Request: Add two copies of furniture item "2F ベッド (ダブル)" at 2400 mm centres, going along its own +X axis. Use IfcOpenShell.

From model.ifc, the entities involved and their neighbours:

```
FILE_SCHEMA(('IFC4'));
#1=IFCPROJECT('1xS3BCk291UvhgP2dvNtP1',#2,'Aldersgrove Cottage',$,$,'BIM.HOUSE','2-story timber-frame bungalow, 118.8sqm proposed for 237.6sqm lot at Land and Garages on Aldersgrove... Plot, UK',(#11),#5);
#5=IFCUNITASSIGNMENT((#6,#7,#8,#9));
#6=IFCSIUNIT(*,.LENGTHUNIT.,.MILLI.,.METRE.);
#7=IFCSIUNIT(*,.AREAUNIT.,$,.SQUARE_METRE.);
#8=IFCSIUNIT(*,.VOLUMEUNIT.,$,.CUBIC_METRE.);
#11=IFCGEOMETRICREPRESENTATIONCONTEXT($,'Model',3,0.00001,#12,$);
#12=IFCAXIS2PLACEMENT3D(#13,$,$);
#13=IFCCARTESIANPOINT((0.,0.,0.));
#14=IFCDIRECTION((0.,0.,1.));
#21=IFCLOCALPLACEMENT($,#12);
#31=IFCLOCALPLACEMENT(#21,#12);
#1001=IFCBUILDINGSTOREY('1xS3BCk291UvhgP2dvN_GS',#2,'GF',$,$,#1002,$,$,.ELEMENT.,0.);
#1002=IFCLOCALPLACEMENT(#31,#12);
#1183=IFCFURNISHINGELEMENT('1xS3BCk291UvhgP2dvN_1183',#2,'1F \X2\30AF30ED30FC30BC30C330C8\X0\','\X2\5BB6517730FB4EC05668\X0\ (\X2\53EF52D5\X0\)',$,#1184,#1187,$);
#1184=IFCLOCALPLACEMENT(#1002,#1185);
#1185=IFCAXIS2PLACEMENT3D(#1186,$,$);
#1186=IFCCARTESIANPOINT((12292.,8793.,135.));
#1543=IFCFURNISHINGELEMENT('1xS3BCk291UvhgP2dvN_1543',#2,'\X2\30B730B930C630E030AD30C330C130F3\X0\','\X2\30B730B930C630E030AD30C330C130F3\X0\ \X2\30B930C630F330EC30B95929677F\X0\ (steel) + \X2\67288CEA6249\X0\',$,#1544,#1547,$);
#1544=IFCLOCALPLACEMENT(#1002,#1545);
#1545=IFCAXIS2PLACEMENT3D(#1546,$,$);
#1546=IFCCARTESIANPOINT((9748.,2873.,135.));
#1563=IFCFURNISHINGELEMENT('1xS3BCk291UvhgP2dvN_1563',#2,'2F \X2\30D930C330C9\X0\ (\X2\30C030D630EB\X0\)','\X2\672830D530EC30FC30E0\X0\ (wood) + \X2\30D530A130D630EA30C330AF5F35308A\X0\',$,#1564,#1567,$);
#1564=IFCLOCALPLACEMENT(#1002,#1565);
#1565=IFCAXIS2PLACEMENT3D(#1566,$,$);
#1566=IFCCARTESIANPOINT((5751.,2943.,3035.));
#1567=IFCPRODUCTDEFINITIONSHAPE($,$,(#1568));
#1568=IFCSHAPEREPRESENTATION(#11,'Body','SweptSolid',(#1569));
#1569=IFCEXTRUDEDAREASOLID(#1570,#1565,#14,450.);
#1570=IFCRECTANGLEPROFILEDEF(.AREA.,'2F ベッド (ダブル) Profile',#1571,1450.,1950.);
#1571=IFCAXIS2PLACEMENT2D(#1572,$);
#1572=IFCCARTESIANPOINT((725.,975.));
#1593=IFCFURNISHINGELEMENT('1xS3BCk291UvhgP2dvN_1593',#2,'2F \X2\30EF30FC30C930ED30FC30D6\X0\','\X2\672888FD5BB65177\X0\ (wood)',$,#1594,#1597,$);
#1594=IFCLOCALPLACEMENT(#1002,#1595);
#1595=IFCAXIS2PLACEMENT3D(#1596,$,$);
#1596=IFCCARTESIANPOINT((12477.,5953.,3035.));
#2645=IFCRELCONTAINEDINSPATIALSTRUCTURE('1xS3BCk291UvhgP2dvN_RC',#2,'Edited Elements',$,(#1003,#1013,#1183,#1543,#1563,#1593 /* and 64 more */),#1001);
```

```python
import ifcopenshell
import ifcopenshell.api.geometry
import ifcopenshell.api.root
import ifcopenshell.util.element
import ifcopenshell.util.placement

model = ifcopenshell.open("model.ifc")


def reuse_history(source, copy):
    """copy_class also copies each property set's owner history, people and application; keep the originals."""
    for rel in copy.IsDefinedBy:
        if rel.is_a("IfcRelDefinesByProperties") and (history := rel.RelatingPropertyDefinition.OwnerHistory):
            rel.RelatingPropertyDefinition.OwnerHistory = source.OwnerHistory
            ifcopenshell.util.element.remove_deep2(model, history)


source = model.by_guid("1xS3BCk291UvhgP2dvN_1563")
base = ifcopenshell.util.placement.get_local_placement(source.ObjectPlacement)
step = base[:3, 0] * 2400.0

for i in range(1, 3):
    copy = ifcopenshell.api.root.copy_class(model, product=source)
    copy.Representation = ifcopenshell.util.element.copy_deep(
        model, source.Representation, exclude=["IfcGeometricRepresentationContext", "IfcRepresentationMap"]
    )
    reuse_history(source, copy)
    matrix = base.copy()
    matrix[:3, 3] += i * step
    print("added at", matrix[:3, 3].round(3) + 0.0)
    ifcopenshell.api.geometry.edit_object_placement(model, product=copy, matrix=matrix, is_si=False)

model.write("model_rev.ifc")
```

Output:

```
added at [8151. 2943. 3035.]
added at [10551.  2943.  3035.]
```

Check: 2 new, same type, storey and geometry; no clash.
